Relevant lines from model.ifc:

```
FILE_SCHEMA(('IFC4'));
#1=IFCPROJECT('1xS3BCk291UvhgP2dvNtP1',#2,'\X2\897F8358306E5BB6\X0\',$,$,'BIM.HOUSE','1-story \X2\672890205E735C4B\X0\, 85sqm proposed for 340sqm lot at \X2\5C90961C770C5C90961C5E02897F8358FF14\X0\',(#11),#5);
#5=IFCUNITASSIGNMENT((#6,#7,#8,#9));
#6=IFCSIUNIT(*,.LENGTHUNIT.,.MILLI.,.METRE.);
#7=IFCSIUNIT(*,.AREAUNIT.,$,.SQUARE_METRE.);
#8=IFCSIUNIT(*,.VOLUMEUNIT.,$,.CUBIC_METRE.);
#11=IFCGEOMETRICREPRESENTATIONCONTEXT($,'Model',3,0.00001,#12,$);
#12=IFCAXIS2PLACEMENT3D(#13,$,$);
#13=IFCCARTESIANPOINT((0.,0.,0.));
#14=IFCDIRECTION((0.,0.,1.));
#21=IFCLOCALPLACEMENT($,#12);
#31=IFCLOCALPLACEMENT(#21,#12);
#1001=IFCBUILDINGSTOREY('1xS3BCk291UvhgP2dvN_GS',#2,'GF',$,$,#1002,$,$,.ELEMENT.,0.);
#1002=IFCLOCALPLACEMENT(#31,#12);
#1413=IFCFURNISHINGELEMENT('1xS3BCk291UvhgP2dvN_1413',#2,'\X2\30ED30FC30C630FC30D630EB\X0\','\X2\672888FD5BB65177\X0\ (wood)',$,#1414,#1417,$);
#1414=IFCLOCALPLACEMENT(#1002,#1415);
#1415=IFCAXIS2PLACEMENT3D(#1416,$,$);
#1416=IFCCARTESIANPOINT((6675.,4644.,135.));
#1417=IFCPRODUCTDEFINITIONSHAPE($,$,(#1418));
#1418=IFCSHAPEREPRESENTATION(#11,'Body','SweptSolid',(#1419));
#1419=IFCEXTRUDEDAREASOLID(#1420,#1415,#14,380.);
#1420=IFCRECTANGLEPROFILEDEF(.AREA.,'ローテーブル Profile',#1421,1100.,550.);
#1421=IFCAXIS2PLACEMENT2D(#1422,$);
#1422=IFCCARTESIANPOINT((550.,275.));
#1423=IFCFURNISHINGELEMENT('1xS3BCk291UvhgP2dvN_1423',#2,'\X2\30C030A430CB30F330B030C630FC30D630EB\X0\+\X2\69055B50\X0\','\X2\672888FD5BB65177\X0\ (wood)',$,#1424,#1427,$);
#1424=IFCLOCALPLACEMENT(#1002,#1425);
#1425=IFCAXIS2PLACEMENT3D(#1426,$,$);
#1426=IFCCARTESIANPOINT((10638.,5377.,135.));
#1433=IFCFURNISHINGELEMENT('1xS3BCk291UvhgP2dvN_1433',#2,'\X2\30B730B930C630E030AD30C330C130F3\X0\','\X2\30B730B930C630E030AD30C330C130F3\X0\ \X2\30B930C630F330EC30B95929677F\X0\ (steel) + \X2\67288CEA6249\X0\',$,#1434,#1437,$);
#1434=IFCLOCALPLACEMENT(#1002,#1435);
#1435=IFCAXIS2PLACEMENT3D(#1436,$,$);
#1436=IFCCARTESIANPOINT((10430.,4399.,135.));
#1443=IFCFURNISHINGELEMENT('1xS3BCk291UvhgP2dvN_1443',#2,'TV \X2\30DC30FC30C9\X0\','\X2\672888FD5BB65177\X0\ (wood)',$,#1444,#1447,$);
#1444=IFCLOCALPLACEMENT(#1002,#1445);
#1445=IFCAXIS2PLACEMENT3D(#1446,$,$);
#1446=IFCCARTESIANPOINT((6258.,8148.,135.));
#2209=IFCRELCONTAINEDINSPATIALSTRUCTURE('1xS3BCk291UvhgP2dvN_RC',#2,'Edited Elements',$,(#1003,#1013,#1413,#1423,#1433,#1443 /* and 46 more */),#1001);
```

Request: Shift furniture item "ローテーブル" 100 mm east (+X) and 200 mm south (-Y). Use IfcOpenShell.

```python
import ifcopenshell
import ifcopenshell.api.geometry
import ifcopenshell.util.placement
import ifcopenshell.util.unit

model = ifcopenshell.open("model.ifc")
unit_scale = ifcopenshell.util.unit.calculate_unit_scale(model)

item = model.by_guid("1xS3BCk291UvhgP2dvN_1413")
matrix = ifcopenshell.util.placement.get_local_placement(item.ObjectPlacement)
matrix[0, 3] += 0.1 / unit_scale
matrix[1, 3] -= 0.2 / unit_scale
ifcopenshell.api.geometry.edit_object_placement(model, product=item, matrix=matrix, is_si=False)

print(ifcopenshell.util.placement.get_local_placement(item.ObjectPlacement).round(3) + 0.0)

model.write("model_v2.ifc")
```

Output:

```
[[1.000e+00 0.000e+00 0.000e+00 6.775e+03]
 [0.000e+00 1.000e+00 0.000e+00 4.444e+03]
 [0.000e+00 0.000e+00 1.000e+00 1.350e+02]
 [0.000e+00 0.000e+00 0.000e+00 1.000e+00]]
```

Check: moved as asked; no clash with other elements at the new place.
